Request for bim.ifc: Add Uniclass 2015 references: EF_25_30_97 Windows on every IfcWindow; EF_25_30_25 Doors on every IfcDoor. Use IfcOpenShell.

First a look at what the model holds.

```python
import ifcopenshell

model = ifcopenshell.open("bim.ifc")
print(model.schema)
print("classifications:", [c.Name for c in model.by_type("IfcClassification")])
for ifc_class in ("IfcDoor", "IfcRoof", "IfcStair", "IfcWall", "IfcWindow"):
    print(ifc_class, len(model.by_type(ifc_class)))
```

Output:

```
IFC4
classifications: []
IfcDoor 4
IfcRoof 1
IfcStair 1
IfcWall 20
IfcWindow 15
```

```python
import ifcopenshell
import ifcopenshell.api.classification

model = ifcopenshell.open("bim.ifc")

system = ifcopenshell.api.classification.add_classification(model, classification="Uniclass 2015")

codes = {
    "IfcWindow": ("EF_25_30_97", "Windows"),
    "IfcDoor": ("EF_25_30_25", "Doors"),
}
for ifc_class, (code, name) in codes.items():
    products = model.by_type(ifc_class)
    ifcopenshell.api.classification.add_reference(
        model, products=products, classification=system, identification=code, name=name
    )
    print(code, len(products))

model.write("bim_rev.ifc")
```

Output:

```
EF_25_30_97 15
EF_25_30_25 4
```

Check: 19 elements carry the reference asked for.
